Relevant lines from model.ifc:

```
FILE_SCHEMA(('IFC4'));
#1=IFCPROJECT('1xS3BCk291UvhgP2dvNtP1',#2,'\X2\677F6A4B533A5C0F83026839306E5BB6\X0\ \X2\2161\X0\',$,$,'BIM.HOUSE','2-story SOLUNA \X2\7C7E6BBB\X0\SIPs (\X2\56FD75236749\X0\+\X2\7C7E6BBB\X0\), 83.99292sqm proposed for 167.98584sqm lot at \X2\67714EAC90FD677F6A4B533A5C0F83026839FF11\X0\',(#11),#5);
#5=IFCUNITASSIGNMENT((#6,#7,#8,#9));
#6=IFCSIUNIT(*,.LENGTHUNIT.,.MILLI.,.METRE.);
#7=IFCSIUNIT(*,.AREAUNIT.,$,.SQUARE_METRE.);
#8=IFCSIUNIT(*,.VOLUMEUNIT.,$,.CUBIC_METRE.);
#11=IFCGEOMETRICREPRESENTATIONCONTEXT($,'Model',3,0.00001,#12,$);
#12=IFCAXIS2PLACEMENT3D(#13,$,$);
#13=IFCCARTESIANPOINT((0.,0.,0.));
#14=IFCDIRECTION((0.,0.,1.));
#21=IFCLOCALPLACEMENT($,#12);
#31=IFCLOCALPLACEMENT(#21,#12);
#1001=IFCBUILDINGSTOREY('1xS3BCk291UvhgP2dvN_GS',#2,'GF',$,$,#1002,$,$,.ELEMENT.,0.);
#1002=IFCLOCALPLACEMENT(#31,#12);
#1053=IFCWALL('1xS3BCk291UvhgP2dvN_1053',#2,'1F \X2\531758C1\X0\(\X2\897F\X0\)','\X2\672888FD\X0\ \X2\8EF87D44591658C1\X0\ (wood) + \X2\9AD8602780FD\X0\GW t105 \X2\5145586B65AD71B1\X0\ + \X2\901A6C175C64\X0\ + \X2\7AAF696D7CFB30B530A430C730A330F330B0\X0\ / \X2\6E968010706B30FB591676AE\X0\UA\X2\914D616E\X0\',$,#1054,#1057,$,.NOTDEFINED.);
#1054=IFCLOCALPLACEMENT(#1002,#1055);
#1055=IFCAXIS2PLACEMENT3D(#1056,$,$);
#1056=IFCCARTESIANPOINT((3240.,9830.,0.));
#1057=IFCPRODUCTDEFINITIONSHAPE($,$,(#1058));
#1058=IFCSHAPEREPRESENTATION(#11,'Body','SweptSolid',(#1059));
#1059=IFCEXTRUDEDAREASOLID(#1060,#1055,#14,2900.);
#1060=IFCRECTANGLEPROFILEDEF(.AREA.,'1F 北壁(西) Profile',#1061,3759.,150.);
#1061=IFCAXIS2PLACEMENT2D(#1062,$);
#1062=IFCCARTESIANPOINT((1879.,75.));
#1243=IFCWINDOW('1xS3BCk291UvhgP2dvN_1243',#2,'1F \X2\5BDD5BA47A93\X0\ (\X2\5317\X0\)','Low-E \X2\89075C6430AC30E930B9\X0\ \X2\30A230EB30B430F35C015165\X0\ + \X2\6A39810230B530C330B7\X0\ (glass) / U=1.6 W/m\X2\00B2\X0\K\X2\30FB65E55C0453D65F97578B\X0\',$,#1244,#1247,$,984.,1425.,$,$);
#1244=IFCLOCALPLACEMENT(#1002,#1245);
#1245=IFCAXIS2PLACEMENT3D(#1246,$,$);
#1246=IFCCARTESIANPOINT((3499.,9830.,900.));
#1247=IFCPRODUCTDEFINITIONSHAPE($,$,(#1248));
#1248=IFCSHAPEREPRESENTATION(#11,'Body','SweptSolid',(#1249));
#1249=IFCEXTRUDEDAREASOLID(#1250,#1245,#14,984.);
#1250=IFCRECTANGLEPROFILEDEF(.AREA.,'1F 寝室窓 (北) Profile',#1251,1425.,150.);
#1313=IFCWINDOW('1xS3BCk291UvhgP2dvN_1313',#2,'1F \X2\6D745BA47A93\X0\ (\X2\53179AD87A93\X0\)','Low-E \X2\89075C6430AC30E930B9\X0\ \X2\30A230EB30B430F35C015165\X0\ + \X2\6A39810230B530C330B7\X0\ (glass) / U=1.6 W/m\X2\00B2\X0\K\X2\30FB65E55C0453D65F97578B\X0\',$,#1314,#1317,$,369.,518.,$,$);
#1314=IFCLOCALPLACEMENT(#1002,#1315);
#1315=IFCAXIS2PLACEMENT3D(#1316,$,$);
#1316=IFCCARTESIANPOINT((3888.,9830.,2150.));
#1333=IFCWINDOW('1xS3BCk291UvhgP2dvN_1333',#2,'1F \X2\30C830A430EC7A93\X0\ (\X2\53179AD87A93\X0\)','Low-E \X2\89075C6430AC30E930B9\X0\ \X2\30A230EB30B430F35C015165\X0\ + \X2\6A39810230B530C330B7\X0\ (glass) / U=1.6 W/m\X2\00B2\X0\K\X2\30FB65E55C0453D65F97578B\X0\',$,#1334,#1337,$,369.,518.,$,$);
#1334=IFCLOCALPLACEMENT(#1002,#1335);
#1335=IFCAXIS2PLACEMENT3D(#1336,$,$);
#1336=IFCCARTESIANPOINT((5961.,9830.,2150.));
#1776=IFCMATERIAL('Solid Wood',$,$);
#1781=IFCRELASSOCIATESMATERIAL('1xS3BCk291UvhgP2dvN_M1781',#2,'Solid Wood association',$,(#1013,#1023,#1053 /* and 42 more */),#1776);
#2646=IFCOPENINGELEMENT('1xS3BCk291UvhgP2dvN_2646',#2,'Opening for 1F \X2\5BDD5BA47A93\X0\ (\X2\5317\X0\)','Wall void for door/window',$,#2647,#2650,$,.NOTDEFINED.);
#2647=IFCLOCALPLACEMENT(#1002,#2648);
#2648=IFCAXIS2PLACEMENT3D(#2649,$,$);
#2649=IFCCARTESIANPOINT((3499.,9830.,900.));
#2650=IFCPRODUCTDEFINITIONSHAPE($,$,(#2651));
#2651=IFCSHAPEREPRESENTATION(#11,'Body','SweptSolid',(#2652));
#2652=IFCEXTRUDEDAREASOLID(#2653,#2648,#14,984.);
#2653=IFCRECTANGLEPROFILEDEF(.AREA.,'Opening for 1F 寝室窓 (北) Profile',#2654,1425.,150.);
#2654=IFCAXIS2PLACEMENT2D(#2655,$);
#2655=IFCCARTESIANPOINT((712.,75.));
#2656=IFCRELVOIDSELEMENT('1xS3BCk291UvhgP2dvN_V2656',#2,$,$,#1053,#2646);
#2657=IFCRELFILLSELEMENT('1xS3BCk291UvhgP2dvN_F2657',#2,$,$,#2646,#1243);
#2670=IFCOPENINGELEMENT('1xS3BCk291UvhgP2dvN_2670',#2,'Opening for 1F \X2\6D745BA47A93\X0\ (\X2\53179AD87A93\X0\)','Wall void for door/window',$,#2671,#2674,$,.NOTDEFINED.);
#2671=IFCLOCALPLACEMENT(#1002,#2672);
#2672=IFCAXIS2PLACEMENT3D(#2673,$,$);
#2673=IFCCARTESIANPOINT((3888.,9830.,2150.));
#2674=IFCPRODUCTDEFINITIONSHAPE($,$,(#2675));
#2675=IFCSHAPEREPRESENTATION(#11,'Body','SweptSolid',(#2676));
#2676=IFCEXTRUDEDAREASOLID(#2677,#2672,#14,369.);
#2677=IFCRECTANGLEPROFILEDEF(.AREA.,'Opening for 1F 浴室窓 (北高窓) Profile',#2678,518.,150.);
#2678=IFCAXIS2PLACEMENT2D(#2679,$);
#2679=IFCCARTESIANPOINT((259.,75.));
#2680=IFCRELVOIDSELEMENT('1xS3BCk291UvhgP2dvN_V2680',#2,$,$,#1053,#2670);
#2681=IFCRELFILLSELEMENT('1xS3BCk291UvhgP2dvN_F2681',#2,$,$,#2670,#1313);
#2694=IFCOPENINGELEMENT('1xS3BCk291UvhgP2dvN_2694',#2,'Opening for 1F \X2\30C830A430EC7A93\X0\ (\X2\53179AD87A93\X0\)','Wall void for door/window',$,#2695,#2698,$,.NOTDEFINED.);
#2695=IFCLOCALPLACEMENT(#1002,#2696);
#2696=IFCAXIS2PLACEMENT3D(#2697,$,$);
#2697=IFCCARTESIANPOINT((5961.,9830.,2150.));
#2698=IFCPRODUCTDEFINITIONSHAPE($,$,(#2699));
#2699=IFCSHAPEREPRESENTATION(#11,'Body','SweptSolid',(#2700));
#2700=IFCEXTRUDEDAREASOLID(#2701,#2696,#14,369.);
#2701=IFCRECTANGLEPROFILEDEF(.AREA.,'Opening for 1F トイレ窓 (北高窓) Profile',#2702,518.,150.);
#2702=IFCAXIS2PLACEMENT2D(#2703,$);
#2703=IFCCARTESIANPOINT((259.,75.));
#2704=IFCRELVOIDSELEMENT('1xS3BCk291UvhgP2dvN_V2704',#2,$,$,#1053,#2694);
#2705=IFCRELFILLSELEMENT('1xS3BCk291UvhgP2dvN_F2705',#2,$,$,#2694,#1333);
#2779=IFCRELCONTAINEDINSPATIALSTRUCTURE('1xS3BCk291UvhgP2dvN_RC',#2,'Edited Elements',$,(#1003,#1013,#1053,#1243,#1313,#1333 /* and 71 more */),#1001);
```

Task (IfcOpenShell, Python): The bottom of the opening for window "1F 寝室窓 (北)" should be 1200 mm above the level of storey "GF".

```python
import numpy as np
import ifcopenshell
import ifcopenshell.api.geometry
import ifcopenshell.geom
import ifcopenshell.util.element
import ifcopenshell.util.placement
import ifcopenshell.util.shape
import ifcopenshell.util.unit

model = ifcopenshell.open("model.ifc")
unit_scale = ifcopenshell.util.unit.calculate_unit_scale(model)

window = model.by_guid("1xS3BCk291UvhgP2dvN_1243")
opening = window.FillsVoids[0].RelatingOpeningElement
storey = ifcopenshell.util.element.get_container(window, ifc_class="IfcBuildingStorey")
level = ifcopenshell.util.placement.get_local_placement(storey.ObjectPlacement)[2, 3]

# The opening's origin need not be at the sill, so measure its lowest point.
shape = ifcopenshell.geom.create_shape(ifcopenshell.geom.settings(), opening)
bottom = ifcopenshell.util.shape.get_shape_bottom_elevation(shape, shape.geometry) / unit_scale
dz = level + 1.2 / unit_scale - bottom

shift = np.array([0.0, 0.0, dz])
# The window is not placed relative to its opening, so move both.
for product in (opening, window):
    matrix = ifcopenshell.util.placement.get_local_placement(product.ObjectPlacement)
    matrix[:3, 3] += shift
    ifcopenshell.api.geometry.edit_object_placement(model, product=product, matrix=matrix, is_si=False)

print(f"moved by {dz * unit_scale:+.3f} m")

model.write("model_edited.ifc")
```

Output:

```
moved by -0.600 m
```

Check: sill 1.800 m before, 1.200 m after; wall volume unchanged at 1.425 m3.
